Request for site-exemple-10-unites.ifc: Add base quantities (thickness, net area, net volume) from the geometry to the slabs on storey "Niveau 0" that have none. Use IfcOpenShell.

First a look at what the model holds.

```python
import ifcopenshell
import ifcopenshell.util.element
import ifcopenshell.util.unit

model = ifcopenshell.open("site-exemple-10-unites.ifc")
print(model.schema)
for unit_type in ("LENGTHUNIT", "AREAUNIT", "VOLUMEUNIT"):
    print(unit_type, ifcopenshell.util.unit.calculate_unit_scale(model, unit_type))
storey = next(s for s in model.by_type("IfcBuildingStorey") if s.Name == "Niveau 0")
slabs = [e for e in ifcopenshell.util.element.get_decomposition(storey) if e.is_a("IfcSlab")]
for e in sorted(slabs, key=lambda e: e.id()):
    print(e.id(), e.is_a(), e.Name, list(ifcopenshell.util.element.get_psets(e, qtos_only=True)), sep=" | ")
```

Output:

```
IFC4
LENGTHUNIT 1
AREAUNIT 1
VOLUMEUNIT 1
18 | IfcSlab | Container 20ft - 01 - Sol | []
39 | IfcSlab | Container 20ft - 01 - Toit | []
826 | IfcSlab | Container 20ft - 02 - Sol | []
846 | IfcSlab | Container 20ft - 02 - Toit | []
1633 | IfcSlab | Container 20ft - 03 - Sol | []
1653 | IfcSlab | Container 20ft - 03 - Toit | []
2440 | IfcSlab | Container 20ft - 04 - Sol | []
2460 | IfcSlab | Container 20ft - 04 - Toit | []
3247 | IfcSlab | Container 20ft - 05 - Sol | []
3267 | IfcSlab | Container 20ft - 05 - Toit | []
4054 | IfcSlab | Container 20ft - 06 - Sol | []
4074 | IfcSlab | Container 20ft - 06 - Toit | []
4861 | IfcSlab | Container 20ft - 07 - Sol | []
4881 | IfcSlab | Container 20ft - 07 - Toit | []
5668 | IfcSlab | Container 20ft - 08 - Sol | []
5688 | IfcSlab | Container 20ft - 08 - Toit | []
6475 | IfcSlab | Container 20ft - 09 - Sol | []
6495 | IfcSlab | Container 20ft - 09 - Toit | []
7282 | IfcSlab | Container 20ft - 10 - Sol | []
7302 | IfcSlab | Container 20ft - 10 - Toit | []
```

```python
import ifcopenshell
import ifcopenshell.api.pset
import ifcopenshell.geom
import ifcopenshell.util.element
import ifcopenshell.util.shape
import ifcopenshell.util.unit

model = ifcopenshell.open("site-exemple-10-unites.ifc")
unit_scale = ifcopenshell.util.unit.calculate_unit_scale(model)
area_scale = ifcopenshell.util.unit.calculate_unit_scale(model, "AREAUNIT")
volume_scale = ifcopenshell.util.unit.calculate_unit_scale(model, "VOLUMEUNIT")
settings = ifcopenshell.geom.settings()

storey = next(s for s in model.by_type("IfcBuildingStorey") if s.Name == "Niveau 0")
slabs = [e for e in ifcopenshell.util.element.get_decomposition(storey) if e.is_a("IfcSlab")]

for e in sorted(slabs, key=lambda e: e.id()):
    if ifcopenshell.util.element.get_psets(e, qtos_only=True, should_inherit=False):
        continue
    # Geometry comes back in metres, in the element's own axes.
    shape = ifcopenshell.geom.create_shape(settings, e)
    values = {
        "Width": ifcopenshell.util.shape.get_z(shape.geometry) / unit_scale,
        "NetArea": ifcopenshell.util.shape.get_footprint_area(shape.geometry) / area_scale,
        "NetVolume": ifcopenshell.util.shape.get_volume(shape.geometry) / volume_scale,
    }
    qto = ifcopenshell.api.pset.add_qto(model, product=e, name="Qto_SlabBaseQuantities")
    ifcopenshell.api.pset.edit_qto(model, qto=qto, properties=values)
    print(e.id(), {k: round(v, 3) for k, v in values.items()})

model.write("site-exemple-10-unites_updated.ifc")
```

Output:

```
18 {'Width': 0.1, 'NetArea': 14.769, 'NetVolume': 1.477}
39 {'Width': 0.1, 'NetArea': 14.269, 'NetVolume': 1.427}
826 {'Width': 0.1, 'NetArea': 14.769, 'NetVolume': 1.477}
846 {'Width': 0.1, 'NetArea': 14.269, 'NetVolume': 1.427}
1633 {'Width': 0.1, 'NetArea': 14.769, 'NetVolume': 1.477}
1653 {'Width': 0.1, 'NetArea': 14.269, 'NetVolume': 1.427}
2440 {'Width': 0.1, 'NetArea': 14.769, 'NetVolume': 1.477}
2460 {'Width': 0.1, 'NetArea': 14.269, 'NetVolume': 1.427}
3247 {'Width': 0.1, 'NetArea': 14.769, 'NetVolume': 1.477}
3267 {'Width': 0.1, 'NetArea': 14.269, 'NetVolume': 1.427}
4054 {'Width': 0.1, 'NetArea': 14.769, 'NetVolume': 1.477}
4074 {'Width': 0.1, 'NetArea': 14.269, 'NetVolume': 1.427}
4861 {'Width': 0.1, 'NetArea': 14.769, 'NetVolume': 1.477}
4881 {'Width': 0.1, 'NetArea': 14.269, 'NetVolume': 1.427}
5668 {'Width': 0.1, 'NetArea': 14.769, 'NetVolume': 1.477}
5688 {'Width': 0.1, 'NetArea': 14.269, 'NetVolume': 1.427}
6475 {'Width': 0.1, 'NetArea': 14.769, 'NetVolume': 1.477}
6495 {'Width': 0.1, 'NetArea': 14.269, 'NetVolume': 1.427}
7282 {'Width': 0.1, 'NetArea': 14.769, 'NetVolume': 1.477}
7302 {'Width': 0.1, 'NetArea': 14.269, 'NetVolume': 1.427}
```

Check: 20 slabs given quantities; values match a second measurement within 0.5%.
